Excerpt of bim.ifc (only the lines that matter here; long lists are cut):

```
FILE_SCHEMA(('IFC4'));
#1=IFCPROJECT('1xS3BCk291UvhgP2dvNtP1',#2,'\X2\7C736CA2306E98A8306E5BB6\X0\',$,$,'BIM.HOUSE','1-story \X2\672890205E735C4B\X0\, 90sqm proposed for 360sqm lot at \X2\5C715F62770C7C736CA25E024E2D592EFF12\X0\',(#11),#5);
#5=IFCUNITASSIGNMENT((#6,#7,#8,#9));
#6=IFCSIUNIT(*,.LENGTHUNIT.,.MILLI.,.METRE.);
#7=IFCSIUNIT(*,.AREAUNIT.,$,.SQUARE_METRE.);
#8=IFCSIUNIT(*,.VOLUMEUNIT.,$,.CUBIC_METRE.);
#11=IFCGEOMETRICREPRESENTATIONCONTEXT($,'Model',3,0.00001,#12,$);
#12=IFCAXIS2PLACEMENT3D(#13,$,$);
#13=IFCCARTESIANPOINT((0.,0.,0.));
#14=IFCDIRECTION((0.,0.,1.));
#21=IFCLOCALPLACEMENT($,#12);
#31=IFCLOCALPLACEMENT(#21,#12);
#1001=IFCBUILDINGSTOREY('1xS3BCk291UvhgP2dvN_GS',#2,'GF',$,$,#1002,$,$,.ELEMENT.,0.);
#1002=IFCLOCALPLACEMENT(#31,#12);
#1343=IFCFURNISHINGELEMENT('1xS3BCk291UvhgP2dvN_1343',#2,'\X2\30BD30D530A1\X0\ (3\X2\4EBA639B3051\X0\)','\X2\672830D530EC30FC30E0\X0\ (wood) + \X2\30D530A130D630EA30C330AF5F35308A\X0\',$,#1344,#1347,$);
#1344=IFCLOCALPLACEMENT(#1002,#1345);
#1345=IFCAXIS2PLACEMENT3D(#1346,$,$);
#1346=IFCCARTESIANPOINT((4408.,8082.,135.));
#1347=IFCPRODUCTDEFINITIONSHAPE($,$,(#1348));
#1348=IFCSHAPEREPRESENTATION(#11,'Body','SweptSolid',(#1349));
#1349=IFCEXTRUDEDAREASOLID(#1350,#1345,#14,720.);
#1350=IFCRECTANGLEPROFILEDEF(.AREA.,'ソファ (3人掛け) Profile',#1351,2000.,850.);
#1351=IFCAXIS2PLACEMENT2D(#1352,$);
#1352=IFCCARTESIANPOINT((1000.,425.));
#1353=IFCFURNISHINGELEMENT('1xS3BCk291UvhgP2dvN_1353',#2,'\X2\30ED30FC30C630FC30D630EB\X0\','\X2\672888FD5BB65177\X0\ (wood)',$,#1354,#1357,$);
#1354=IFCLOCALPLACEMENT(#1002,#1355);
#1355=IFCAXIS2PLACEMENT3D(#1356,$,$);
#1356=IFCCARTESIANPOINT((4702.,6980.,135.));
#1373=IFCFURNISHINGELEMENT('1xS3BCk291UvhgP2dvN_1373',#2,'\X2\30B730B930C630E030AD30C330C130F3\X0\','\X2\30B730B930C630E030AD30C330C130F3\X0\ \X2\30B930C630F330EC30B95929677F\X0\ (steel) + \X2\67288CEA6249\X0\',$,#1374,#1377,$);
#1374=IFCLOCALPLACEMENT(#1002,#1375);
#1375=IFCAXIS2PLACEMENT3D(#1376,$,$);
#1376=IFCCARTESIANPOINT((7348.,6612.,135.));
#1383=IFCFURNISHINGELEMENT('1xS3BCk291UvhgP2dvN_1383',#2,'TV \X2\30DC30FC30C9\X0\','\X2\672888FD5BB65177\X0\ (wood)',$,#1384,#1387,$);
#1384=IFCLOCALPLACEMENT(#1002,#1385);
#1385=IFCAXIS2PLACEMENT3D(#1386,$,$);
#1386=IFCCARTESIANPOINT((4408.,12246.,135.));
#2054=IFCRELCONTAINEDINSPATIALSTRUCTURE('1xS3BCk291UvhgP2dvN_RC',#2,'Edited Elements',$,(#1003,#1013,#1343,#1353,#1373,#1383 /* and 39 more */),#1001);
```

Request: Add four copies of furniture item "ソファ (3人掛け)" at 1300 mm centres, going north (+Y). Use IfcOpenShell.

```python
import numpy as np
import ifcopenshell
import ifcopenshell.api.geometry
import ifcopenshell.api.root
import ifcopenshell.util.element
import ifcopenshell.util.placement
import ifcopenshell.util.unit

model = ifcopenshell.open("bim.ifc")
unit_scale = ifcopenshell.util.unit.calculate_unit_scale(model)


def reuse_history(source, copy):
    """copy_class also copies each property set's owner history, people and application; keep the originals."""
    for rel in copy.IsDefinedBy:
        if rel.is_a("IfcRelDefinesByProperties") and (history := rel.RelatingPropertyDefinition.OwnerHistory):
            rel.RelatingPropertyDefinition.OwnerHistory = source.OwnerHistory
            ifcopenshell.util.element.remove_deep2(model, history)


source = model.by_guid("1xS3BCk291UvhgP2dvN_1343")
base = ifcopenshell.util.placement.get_local_placement(source.ObjectPlacement)
step = np.array([0.0, 1.0, 0.0]) * 1.3 / unit_scale

for i in range(1, 5):
    copy = ifcopenshell.api.root.copy_class(model, product=source)
    copy.Representation = ifcopenshell.util.element.copy_deep(
        model, source.Representation, exclude=["IfcGeometricRepresentationContext", "IfcRepresentationMap"]
    )
    reuse_history(source, copy)
    matrix = base.copy()
    matrix[:3, 3] += i * step
    print("added at", matrix[:3, 3].round(3) + 0.0)
    ifcopenshell.api.geometry.edit_object_placement(model, product=copy, matrix=matrix, is_si=False)

model.write("bim_edited.ifc")
```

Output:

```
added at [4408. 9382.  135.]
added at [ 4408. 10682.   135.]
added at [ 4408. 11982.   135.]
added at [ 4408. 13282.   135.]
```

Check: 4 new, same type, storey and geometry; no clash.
